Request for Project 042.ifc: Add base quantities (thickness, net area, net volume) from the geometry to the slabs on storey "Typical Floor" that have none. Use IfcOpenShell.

First a look at what the model holds.

```python
import ifcopenshell
import ifcopenshell.util.element
import ifcopenshell.util.unit

model = ifcopenshell.open("Project 042.ifc")
print(model.schema)
for unit_type in ("LENGTHUNIT", "AREAUNIT", "VOLUMEUNIT"):
    print(unit_type, ifcopenshell.util.unit.calculate_unit_scale(model, unit_type))
storey = next(s for s in model.by_type("IfcBuildingStorey") if s.Name == "Typical Floor")
slabs = [e for e in ifcopenshell.util.element.get_decomposition(storey) if e.is_a("IfcSlab")]
for e in sorted(slabs, key=lambda e: e.id()):
    print(e.id(), e.is_a(), e.Name, list(ifcopenshell.util.element.get_psets(e, qtos_only=True)), sep=" | ")
```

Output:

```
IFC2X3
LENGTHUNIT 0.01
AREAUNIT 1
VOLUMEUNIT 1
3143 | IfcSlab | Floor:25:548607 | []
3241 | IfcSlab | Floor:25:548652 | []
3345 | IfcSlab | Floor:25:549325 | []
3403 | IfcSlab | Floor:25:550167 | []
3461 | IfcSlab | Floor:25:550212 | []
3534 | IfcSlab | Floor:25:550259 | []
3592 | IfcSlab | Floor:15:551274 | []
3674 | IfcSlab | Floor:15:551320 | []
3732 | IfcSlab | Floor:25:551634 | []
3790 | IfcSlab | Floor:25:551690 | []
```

```python
import ifcopenshell
import ifcopenshell.api.pset
import ifcopenshell.geom
import ifcopenshell.util.element
import ifcopenshell.util.shape
import ifcopenshell.util.unit

model = ifcopenshell.open("Project 042.ifc")
unit_scale = ifcopenshell.util.unit.calculate_unit_scale(model)
area_scale = ifcopenshell.util.unit.calculate_unit_scale(model, "AREAUNIT")
volume_scale = ifcopenshell.util.unit.calculate_unit_scale(model, "VOLUMEUNIT")
settings = ifcopenshell.geom.settings()

storey = next(s for s in model.by_type("IfcBuildingStorey") if s.Name == "Typical Floor")
slabs = [e for e in ifcopenshell.util.element.get_decomposition(storey) if e.is_a("IfcSlab")]

for e in sorted(slabs, key=lambda e: e.id()):
    if ifcopenshell.util.element.get_psets(e, qtos_only=True, should_inherit=False):
        continue
    # Geometry comes back in metres, in the element's own axes.
    shape = ifcopenshell.geom.create_shape(settings, e)
    values = {
        "Width": ifcopenshell.util.shape.get_z(shape.geometry) / unit_scale,
        "NetArea": ifcopenshell.util.shape.get_footprint_area(shape.geometry) / area_scale,
        "NetVolume": ifcopenshell.util.shape.get_volume(shape.geometry) / volume_scale,
    }
    qto = ifcopenshell.api.pset.add_qto(model, product=e, name="BaseQuantities")
    ifcopenshell.api.pset.edit_qto(model, qto=qto, properties=values)
    print(e.id(), {k: round(v, 3) for k, v in values.items()})

model.write("Project 042_updated.ifc")
```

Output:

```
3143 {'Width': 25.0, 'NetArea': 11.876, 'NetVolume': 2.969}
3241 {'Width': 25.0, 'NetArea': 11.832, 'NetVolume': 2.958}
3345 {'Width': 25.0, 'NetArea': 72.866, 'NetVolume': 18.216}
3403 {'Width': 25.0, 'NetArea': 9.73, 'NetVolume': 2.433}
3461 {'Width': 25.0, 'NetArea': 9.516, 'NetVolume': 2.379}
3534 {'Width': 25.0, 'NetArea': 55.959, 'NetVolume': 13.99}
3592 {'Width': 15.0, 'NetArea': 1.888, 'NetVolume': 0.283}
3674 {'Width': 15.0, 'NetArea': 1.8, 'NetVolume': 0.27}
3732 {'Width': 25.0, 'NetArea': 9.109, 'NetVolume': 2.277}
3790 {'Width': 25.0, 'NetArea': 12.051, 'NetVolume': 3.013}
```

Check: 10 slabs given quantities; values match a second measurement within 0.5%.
